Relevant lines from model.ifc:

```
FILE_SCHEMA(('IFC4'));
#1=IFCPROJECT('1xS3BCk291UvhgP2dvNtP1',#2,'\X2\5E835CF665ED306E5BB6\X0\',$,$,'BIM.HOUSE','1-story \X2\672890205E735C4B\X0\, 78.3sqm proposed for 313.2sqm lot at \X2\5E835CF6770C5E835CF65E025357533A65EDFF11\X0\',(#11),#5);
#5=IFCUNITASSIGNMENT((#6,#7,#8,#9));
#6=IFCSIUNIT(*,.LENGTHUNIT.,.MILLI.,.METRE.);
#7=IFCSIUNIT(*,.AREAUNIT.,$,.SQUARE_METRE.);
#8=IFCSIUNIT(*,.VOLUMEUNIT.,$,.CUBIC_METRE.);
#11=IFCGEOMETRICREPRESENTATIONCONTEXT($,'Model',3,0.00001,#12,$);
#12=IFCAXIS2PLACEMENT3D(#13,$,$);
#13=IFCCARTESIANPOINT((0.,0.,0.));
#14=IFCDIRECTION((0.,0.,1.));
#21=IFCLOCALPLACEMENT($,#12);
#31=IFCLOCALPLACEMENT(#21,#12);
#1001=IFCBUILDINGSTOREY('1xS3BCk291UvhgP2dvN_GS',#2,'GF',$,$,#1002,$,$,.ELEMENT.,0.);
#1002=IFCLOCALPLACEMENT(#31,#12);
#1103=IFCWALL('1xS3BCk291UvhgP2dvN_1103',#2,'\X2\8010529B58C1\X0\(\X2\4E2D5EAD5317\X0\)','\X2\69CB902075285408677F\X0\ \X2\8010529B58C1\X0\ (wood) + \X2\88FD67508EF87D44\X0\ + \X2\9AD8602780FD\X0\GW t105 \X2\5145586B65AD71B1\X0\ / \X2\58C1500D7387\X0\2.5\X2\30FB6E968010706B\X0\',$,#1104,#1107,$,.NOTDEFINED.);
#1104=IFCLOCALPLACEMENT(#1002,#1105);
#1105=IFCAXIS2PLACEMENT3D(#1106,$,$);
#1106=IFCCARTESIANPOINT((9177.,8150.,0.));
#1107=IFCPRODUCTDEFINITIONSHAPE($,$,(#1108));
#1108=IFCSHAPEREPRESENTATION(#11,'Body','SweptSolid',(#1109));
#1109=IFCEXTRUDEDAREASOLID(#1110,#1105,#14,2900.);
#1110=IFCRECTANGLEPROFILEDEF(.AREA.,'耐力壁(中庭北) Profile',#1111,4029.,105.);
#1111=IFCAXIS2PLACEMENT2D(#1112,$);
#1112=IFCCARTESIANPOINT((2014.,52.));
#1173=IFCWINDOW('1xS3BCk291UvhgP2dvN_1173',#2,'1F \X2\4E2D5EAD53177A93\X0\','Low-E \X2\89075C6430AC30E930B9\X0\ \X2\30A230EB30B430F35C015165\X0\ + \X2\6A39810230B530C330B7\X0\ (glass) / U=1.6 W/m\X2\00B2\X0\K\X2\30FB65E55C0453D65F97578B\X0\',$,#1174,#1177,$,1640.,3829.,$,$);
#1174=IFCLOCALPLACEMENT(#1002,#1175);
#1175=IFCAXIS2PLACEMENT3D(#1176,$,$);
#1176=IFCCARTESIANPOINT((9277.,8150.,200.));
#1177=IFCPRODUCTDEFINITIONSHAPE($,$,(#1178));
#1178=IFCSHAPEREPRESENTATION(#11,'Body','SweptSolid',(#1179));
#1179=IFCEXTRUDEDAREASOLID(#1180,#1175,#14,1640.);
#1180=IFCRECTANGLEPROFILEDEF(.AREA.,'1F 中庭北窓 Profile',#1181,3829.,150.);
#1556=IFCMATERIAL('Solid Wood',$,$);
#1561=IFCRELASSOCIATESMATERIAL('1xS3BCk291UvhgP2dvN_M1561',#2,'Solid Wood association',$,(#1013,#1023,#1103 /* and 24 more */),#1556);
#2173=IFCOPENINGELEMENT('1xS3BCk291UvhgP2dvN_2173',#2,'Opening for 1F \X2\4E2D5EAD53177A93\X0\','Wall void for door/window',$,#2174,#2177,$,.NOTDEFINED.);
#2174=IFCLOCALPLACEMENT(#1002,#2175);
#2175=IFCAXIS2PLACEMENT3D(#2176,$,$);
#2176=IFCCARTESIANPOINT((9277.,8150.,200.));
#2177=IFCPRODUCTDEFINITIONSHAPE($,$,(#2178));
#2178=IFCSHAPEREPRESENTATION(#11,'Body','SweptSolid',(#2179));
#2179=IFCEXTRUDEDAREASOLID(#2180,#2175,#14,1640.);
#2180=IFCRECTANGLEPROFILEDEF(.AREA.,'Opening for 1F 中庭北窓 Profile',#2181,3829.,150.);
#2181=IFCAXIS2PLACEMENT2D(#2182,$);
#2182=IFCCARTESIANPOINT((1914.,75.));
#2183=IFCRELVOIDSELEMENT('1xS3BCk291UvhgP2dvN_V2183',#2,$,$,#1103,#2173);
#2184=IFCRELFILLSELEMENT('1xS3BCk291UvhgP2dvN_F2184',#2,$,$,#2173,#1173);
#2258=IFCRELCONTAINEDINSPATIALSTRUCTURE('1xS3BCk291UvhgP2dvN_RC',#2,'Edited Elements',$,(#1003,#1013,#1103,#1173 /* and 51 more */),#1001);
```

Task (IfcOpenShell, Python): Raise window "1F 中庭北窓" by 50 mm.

```python
import numpy as np
import ifcopenshell
import ifcopenshell.api.geometry
import ifcopenshell.util.placement
import ifcopenshell.util.unit

model = ifcopenshell.open("model.ifc")
unit_scale = ifcopenshell.util.unit.calculate_unit_scale(model)

window = model.by_guid("1xS3BCk291UvhgP2dvN_1173")
opening = window.FillsVoids[0].RelatingOpeningElement
dz = 50.0

shift = np.array([0.0, 0.0, dz])
# The window is not placed relative to its opening, so move both.
for product in (opening, window):
    matrix = ifcopenshell.util.placement.get_local_placement(product.ObjectPlacement)
    matrix[:3, 3] += shift
    ifcopenshell.api.geometry.edit_object_placement(model, product=product, matrix=matrix, is_si=False)

print(f"moved by {dz * unit_scale:+.3f} m")

model.write("model_edited.ifc")
```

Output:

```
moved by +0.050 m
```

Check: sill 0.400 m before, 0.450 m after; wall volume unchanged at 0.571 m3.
